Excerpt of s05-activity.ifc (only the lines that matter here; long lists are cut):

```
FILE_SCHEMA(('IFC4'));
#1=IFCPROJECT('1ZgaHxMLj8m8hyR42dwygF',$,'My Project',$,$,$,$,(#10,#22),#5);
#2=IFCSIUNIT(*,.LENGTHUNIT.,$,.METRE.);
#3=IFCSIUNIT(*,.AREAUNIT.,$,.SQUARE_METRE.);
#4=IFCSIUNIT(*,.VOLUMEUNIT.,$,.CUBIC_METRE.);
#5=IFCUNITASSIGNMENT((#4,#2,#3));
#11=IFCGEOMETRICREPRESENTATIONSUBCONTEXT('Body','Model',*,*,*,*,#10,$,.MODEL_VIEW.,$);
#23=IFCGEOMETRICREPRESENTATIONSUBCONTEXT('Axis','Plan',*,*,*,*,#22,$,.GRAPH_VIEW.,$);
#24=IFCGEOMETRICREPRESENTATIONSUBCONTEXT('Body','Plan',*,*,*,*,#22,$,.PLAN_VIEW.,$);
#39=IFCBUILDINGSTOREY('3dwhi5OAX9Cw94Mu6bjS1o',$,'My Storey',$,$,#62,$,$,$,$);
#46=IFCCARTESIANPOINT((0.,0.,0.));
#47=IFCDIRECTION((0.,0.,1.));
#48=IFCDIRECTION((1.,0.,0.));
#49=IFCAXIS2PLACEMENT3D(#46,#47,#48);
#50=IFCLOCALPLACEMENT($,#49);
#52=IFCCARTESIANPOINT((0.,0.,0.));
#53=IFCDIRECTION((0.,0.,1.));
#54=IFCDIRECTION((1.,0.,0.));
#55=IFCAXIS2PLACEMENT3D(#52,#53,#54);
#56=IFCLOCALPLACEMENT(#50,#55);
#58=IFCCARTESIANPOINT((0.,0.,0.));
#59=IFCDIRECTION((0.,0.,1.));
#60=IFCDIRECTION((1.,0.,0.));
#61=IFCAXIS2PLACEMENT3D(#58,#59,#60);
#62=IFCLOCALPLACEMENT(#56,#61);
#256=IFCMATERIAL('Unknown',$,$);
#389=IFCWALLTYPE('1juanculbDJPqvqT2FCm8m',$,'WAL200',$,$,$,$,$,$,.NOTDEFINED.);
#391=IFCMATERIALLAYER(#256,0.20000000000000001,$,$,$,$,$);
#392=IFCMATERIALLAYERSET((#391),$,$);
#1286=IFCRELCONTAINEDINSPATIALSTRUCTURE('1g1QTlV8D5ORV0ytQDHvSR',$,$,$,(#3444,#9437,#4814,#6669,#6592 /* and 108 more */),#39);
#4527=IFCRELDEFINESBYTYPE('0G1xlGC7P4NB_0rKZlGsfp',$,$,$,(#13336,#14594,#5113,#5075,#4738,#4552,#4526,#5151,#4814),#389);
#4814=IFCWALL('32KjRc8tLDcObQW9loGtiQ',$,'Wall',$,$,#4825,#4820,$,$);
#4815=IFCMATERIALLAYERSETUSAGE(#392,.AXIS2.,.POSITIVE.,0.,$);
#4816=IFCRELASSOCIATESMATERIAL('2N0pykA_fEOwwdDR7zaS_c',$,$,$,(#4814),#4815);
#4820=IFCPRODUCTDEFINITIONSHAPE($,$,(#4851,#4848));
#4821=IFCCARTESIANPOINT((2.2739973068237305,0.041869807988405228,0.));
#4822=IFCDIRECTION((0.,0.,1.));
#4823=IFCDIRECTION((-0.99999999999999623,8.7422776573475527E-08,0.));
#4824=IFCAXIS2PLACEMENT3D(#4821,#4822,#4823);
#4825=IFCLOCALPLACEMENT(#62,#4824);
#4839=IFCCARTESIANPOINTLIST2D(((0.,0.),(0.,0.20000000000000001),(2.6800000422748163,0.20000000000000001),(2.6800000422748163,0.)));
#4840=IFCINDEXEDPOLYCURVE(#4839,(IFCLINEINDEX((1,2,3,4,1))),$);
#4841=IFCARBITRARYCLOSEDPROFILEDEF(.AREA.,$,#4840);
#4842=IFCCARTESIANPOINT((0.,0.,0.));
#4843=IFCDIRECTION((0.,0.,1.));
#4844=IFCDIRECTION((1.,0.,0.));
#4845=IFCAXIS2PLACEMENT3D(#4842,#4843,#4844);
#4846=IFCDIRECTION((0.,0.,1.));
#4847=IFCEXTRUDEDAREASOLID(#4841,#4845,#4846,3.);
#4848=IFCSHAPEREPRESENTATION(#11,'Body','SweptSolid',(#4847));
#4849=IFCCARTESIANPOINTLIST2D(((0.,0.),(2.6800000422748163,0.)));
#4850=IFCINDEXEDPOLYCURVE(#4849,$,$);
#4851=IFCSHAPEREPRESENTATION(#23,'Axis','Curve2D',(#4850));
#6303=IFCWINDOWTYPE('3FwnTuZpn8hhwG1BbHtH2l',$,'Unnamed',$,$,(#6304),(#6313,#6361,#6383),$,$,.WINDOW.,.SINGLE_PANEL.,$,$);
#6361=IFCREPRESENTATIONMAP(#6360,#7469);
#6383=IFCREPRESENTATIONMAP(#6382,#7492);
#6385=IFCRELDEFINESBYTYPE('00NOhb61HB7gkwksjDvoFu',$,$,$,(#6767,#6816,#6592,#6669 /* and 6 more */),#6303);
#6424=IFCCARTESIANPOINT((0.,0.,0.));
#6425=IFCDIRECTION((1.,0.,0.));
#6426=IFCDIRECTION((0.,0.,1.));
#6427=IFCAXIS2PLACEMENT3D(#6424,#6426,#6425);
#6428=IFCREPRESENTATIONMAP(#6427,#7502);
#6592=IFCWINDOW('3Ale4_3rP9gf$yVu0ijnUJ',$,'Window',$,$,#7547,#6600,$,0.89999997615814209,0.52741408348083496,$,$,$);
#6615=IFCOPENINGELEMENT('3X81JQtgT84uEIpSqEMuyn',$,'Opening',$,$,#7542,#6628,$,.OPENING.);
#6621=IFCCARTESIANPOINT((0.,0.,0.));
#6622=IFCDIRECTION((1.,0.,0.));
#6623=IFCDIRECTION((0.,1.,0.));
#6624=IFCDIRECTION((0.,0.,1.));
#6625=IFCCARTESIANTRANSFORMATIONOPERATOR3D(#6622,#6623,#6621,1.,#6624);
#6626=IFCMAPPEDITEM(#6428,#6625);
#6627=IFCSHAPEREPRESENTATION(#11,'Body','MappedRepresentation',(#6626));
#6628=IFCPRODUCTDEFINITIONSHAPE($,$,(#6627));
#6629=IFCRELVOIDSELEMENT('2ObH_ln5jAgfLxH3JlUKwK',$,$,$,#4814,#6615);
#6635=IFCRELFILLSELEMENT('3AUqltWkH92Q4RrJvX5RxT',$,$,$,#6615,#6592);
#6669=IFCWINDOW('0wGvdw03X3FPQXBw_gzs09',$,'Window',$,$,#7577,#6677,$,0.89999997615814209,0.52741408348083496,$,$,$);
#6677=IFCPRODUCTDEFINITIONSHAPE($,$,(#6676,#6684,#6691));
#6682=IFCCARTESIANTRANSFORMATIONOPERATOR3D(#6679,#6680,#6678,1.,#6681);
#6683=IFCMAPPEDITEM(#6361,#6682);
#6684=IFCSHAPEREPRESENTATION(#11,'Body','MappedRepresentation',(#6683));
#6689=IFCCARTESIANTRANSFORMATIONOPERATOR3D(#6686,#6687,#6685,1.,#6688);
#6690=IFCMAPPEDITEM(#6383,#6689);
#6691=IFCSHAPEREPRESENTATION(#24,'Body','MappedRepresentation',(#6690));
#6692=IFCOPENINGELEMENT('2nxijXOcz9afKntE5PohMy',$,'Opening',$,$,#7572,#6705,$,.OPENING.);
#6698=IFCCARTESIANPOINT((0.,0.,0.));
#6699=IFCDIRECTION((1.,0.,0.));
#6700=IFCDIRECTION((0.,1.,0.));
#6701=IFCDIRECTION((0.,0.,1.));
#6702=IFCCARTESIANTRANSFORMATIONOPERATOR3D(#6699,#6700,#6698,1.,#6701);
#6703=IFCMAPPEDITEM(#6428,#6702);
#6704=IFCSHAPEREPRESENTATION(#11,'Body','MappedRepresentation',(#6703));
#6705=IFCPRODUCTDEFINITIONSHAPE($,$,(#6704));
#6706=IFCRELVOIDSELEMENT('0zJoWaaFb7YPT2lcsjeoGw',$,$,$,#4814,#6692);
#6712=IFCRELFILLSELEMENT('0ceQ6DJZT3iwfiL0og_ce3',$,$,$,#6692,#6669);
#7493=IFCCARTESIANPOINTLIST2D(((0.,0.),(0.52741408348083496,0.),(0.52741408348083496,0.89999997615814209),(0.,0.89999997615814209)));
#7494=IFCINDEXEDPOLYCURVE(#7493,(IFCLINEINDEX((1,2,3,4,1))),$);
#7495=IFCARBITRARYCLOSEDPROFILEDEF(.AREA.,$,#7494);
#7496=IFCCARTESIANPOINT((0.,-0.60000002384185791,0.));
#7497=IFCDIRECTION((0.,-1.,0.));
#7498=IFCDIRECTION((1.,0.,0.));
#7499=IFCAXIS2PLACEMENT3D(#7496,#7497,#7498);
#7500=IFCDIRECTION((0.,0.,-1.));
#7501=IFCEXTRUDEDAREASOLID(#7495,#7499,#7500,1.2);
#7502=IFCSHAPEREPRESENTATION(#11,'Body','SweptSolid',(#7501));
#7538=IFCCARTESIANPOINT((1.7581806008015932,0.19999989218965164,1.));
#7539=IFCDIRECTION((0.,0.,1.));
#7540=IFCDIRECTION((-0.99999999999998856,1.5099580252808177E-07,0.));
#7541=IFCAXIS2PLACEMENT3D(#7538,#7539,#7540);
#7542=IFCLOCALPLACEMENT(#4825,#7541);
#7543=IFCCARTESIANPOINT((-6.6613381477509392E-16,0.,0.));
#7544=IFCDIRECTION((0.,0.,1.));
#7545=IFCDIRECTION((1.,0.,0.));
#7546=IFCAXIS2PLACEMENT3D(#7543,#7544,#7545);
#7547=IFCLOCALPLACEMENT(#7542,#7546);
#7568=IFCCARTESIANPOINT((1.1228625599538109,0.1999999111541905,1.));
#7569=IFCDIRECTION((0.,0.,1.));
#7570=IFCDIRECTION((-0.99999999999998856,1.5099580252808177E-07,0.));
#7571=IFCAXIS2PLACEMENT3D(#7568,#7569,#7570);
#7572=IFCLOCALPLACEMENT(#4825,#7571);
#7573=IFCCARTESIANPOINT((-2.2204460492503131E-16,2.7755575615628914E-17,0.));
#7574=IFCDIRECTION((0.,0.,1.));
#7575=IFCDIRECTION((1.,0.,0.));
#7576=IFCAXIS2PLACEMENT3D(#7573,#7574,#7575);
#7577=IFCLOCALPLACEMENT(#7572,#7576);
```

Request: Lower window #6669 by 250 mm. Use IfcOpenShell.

```python
import numpy as np
import ifcopenshell
import ifcopenshell.api.geometry
import ifcopenshell.util.placement
import ifcopenshell.util.unit

model = ifcopenshell.open("s05-activity.ifc")
unit_scale = ifcopenshell.util.unit.calculate_unit_scale(model)

window = model.by_id(6669)
opening = window.FillsVoids[0].RelatingOpeningElement
dz = -0.25

shift = np.array([0.0, 0.0, dz])
# The window is placed relative to its opening, so it follows when the opening moves.
matrix = ifcopenshell.util.placement.get_local_placement(opening.ObjectPlacement)
matrix[:3, 3] += shift
ifcopenshell.api.geometry.edit_object_placement(
    model, product=opening, matrix=matrix, is_si=False, should_transform_children=True
)

print(f"moved by {dz * unit_scale:+.3f} m")

model.write("s05-activity-out.ifc")
```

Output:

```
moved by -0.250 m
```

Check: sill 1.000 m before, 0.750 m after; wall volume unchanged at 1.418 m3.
